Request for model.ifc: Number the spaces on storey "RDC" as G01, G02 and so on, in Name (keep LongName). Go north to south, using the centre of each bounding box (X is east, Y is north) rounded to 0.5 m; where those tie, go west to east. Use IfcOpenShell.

First a look at what the model holds.

```python
import ifcopenshell
import ifcopenshell.util.element
import ifcopenshell.util.placement

model = ifcopenshell.open("model.ifc")
print(model.schema)
storey = next(s for s in model.by_type("IfcBuildingStorey") if s.Name == "RDC")
spaces = [e for e in ifcopenshell.util.element.get_decomposition(storey) if e.is_a("IfcSpace")]
for e in sorted(spaces, key=lambda e: e.id()):
    origin = ifcopenshell.util.placement.get_local_placement(e.ObjectPlacement)[:3, 3]
    print(e.id(), e.Name, e.LongName, origin.round(2) + 0.0, sep=" | ")
```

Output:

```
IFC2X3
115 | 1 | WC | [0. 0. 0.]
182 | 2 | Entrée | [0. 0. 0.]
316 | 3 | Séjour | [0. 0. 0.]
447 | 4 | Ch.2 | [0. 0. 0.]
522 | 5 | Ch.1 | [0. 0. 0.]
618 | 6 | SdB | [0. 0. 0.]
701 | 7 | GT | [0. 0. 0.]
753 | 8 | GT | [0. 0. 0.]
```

```python
import ifcopenshell
import ifcopenshell.geom
import ifcopenshell.util.element
import ifcopenshell.util.shape

model = ifcopenshell.open("model.ifc")
settings = ifcopenshell.geom.settings()
settings.set("use-world-coords", True)


def centre(element):
    shape = ifcopenshell.geom.create_shape(settings, element)
    return ifcopenshell.util.shape.get_bbox_centroid(shape.geometry)


storey = next(s for s in model.by_type("IfcBuildingStorey") if s.Name == "RDC")
spaces = [e for e in ifcopenshell.util.element.get_decomposition(storey) if e.is_a("IfcSpace")]

# Insertion points can sit at a corner or the storey origin, so sort by the geometry (in metres).
centres = {e: centre(e) for e in spaces}
spaces.sort(key=lambda e: (-round(centres[e][1] / 0.5), centres[e][0]))

for i, e in enumerate(spaces, start=1):
    number = f"G{i:02d}"
    e.Name = number
    print(e.id(), number)

model.write("model_edited.ifc")
```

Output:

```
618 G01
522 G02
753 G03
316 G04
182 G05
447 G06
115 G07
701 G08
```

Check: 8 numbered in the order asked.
